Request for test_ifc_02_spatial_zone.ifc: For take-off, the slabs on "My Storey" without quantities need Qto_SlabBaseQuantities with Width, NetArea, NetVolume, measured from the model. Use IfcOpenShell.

First a look at what the model holds.

```python
import ifcopenshell
import ifcopenshell.util.element
import ifcopenshell.util.unit

model = ifcopenshell.open("test_ifc_02_spatial_zone.ifc")
print(model.schema)
for unit_type in ("LENGTHUNIT", "AREAUNIT", "VOLUMEUNIT"):
    print(unit_type, ifcopenshell.util.unit.calculate_unit_scale(model, unit_type))
storey = next(s for s in model.by_type("IfcBuildingStorey") if s.Name == "My Storey")
slabs = [e for e in ifcopenshell.util.element.get_decomposition(storey) if e.is_a("IfcSlab")]
for e in sorted(slabs, key=lambda e: e.id()):
    print(e.id(), e.is_a(), e.Name, list(ifcopenshell.util.element.get_psets(e, qtos_only=True)), sep=" | ")
```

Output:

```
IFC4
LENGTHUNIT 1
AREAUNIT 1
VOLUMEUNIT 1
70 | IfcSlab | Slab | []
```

```python
import ifcopenshell
import ifcopenshell.api.pset
import ifcopenshell.geom
import ifcopenshell.util.element
import ifcopenshell.util.shape
import ifcopenshell.util.unit

model = ifcopenshell.open("test_ifc_02_spatial_zone.ifc")
unit_scale = ifcopenshell.util.unit.calculate_unit_scale(model)
area_scale = ifcopenshell.util.unit.calculate_unit_scale(model, "AREAUNIT")
volume_scale = ifcopenshell.util.unit.calculate_unit_scale(model, "VOLUMEUNIT")
settings = ifcopenshell.geom.settings()

storey = next(s for s in model.by_type("IfcBuildingStorey") if s.Name == "My Storey")
slabs = [e for e in ifcopenshell.util.element.get_decomposition(storey) if e.is_a("IfcSlab")]

for e in sorted(slabs, key=lambda e: e.id()):
    if ifcopenshell.util.element.get_psets(e, qtos_only=True, should_inherit=False):
        continue
    # Geometry comes back in metres, in the element's own axes.
    shape = ifcopenshell.geom.create_shape(settings, e)
    values = {
        "Width": ifcopenshell.util.shape.get_z(shape.geometry) / unit_scale,
        "NetArea": ifcopenshell.util.shape.get_footprint_area(shape.geometry) / area_scale,
        "NetVolume": ifcopenshell.util.shape.get_volume(shape.geometry) / volume_scale,
    }
    qto = ifcopenshell.api.pset.add_qto(model, product=e, name="Qto_SlabBaseQuantities")
    ifcopenshell.api.pset.edit_qto(model, qto=qto, properties=values)
    print(e.id(), {k: round(v, 3) for k, v in values.items()})

model.write("test_ifc_02_spatial_zone_updated.ifc")
```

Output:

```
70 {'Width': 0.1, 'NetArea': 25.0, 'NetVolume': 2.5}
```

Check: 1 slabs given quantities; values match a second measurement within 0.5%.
